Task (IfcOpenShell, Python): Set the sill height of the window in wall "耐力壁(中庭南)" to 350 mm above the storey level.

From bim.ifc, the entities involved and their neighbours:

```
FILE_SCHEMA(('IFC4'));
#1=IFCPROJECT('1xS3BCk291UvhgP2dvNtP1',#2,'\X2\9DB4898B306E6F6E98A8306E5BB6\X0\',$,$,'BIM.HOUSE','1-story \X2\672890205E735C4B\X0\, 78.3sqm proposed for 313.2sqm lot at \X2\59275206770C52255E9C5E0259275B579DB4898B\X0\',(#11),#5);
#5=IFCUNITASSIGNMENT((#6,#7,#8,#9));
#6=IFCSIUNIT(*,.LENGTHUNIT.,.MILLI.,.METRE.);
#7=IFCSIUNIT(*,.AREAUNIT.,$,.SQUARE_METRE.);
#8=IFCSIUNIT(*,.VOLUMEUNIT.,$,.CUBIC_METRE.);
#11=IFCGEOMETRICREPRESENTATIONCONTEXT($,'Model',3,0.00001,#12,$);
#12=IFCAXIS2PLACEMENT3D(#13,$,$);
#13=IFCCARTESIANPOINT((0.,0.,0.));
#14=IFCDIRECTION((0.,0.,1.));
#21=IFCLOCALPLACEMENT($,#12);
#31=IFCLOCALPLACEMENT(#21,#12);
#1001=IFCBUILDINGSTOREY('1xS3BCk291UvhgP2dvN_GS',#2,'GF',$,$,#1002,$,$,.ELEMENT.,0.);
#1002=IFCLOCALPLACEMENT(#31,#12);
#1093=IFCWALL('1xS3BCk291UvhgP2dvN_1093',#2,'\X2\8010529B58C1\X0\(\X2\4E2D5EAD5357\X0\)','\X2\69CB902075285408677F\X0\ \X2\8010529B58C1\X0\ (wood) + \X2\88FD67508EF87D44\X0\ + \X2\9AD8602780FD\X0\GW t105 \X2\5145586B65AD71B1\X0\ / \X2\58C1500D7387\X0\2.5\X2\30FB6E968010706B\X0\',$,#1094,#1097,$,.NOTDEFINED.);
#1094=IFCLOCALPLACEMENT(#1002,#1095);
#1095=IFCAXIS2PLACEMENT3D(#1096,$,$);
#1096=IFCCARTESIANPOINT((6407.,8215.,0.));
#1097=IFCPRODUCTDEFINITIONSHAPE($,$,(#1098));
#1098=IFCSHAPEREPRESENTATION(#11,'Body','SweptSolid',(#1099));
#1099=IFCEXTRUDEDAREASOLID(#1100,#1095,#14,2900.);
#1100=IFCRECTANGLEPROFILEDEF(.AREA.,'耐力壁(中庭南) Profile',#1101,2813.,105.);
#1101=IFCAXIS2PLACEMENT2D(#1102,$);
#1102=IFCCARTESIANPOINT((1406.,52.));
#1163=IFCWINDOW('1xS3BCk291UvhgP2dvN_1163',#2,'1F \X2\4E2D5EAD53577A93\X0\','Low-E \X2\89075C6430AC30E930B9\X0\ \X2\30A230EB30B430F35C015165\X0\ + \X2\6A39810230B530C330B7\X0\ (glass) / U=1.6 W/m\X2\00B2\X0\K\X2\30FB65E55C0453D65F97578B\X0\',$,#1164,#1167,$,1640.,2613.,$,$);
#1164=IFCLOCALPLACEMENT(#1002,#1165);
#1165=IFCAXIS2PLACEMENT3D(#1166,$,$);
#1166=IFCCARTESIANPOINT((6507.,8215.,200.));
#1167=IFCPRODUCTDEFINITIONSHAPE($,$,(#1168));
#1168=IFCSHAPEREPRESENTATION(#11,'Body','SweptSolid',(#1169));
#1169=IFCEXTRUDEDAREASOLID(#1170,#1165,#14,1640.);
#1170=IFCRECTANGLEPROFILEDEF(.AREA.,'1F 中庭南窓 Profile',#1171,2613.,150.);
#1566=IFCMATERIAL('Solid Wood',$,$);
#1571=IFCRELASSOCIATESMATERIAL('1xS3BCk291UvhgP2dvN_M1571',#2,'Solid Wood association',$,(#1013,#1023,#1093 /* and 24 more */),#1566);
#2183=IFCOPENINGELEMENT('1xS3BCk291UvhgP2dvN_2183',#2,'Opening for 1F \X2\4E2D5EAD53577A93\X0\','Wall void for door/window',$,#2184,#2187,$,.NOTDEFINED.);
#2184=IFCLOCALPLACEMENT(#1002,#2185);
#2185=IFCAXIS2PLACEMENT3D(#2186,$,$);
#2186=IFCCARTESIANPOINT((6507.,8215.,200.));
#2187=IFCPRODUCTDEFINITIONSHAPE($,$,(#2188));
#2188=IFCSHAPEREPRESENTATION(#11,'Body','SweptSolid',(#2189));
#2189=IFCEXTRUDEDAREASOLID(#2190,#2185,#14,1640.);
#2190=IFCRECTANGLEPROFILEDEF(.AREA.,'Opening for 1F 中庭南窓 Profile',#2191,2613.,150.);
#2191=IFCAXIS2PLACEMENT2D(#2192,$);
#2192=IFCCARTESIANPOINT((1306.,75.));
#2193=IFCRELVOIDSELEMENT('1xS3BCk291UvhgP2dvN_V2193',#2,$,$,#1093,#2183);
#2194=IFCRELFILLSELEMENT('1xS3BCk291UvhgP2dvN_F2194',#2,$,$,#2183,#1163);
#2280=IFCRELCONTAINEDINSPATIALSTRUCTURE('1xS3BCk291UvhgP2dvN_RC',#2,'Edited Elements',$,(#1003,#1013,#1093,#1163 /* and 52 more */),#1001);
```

```python
import numpy as np
import ifcopenshell
import ifcopenshell.api.geometry
import ifcopenshell.geom
import ifcopenshell.util.element
import ifcopenshell.util.placement
import ifcopenshell.util.shape
import ifcopenshell.util.unit

model = ifcopenshell.open("bim.ifc")
unit_scale = ifcopenshell.util.unit.calculate_unit_scale(model)

window = model.by_id(1163)
opening = window.FillsVoids[0].RelatingOpeningElement
storey = ifcopenshell.util.element.get_container(window, ifc_class="IfcBuildingStorey")
level = ifcopenshell.util.placement.get_local_placement(storey.ObjectPlacement)[2, 3]

# The opening's origin need not be at the sill, so measure its lowest point.
shape = ifcopenshell.geom.create_shape(ifcopenshell.geom.settings(), opening)
bottom = ifcopenshell.util.shape.get_shape_bottom_elevation(shape, shape.geometry) / unit_scale
dz = level + 0.35 / unit_scale - bottom

shift = np.array([0.0, 0.0, dz])
# The window is not placed relative to its opening, so move both.
for product in (opening, window):
    matrix = ifcopenshell.util.placement.get_local_placement(product.ObjectPlacement)
    matrix[:3, 3] += shift
    ifcopenshell.api.geometry.edit_object_placement(model, product=product, matrix=matrix, is_si=False)

print(f"moved by {dz * unit_scale:+.3f} m")

model.write("bim_updated.ifc")
```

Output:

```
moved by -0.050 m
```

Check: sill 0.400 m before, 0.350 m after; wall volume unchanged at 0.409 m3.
